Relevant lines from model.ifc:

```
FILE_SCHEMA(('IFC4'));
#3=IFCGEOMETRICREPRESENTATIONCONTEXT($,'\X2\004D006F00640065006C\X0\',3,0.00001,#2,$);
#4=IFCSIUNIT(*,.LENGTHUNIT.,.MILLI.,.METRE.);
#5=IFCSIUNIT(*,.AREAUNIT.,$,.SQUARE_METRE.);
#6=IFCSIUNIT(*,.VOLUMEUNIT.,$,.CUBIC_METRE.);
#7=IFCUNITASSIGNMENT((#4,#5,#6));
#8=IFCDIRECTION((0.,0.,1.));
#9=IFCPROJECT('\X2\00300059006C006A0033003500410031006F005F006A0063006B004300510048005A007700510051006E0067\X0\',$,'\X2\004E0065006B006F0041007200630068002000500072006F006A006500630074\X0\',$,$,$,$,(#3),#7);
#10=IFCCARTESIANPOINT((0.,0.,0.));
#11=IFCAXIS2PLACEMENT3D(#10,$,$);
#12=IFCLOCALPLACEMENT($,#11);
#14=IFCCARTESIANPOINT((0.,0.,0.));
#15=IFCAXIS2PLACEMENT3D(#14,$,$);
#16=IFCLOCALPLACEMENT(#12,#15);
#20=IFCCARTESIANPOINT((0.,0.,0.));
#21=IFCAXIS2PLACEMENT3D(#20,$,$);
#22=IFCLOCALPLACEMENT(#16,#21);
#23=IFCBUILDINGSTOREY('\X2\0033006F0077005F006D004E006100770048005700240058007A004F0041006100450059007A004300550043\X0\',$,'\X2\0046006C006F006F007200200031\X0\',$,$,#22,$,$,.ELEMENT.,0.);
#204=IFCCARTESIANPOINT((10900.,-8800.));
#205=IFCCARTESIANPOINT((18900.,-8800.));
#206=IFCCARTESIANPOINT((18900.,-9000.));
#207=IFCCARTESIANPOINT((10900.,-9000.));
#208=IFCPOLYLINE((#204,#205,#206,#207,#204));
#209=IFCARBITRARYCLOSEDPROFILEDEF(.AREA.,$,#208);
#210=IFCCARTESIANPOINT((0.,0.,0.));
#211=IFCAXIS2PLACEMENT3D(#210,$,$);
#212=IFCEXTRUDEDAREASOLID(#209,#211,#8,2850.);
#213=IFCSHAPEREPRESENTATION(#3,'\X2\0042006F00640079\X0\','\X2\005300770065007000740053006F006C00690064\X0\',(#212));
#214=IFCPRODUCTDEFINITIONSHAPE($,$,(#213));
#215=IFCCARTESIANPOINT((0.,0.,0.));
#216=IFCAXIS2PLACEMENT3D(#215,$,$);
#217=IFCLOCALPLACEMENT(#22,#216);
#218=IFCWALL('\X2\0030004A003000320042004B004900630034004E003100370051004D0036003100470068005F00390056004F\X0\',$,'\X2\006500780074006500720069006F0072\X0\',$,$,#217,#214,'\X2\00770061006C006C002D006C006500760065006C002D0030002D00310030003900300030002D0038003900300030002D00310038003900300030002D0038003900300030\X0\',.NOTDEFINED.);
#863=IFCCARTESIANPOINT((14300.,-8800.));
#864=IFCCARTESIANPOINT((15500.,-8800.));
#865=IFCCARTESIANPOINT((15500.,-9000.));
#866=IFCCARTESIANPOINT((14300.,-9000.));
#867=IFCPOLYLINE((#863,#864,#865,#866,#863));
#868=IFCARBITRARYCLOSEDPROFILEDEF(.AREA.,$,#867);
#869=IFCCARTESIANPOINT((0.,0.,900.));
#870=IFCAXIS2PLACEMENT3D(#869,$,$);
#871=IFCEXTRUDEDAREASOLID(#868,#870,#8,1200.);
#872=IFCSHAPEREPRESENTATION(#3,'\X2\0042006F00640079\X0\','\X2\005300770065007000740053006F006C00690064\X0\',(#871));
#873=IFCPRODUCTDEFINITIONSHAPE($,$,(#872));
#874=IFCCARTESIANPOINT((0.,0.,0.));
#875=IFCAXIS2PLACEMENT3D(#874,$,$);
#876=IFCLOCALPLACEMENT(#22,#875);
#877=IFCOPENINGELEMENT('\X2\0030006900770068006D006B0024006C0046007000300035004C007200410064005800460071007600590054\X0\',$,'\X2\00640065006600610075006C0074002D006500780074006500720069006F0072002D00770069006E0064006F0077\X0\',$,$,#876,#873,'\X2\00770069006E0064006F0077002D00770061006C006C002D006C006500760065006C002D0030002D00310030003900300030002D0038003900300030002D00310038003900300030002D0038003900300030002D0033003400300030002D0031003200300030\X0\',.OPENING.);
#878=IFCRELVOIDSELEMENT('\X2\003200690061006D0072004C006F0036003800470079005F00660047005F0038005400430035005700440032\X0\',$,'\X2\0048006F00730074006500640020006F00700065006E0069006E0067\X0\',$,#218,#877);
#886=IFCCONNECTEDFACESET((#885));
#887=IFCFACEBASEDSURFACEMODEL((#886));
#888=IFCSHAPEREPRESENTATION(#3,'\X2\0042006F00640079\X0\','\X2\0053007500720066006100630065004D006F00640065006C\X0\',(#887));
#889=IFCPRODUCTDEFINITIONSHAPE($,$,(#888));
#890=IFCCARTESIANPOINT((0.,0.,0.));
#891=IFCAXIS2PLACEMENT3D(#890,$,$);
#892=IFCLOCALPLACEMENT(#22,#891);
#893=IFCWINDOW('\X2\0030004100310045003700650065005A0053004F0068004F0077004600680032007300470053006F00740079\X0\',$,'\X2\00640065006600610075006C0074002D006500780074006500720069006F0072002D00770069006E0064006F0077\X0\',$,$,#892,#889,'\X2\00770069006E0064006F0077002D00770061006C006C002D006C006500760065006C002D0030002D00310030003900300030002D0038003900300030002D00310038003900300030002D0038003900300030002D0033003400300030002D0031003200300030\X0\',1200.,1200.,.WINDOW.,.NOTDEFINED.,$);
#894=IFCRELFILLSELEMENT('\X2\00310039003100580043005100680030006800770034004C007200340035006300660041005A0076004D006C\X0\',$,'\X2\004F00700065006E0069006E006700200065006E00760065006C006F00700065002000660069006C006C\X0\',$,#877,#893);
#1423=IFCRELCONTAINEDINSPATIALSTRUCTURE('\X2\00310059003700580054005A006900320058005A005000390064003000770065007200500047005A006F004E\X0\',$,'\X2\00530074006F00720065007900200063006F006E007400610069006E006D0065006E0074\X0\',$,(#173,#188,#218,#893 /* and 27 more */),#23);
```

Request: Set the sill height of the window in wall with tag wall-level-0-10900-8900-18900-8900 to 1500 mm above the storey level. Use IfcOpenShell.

```python
import numpy as np
import ifcopenshell
import ifcopenshell.api.geometry
import ifcopenshell.geom
import ifcopenshell.util.element
import ifcopenshell.util.placement
import ifcopenshell.util.shape
import ifcopenshell.util.unit

model = ifcopenshell.open("model.ifc")
unit_scale = ifcopenshell.util.unit.calculate_unit_scale(model)

window = model.by_guid("0A1E7eeZSOhOwFh2sGSoty")
opening = window.FillsVoids[0].RelatingOpeningElement
storey = ifcopenshell.util.element.get_container(window, ifc_class="IfcBuildingStorey")
level = ifcopenshell.util.placement.get_local_placement(storey.ObjectPlacement)[2, 3]

# The opening's origin need not be at the sill, so measure its lowest point.
shape = ifcopenshell.geom.create_shape(ifcopenshell.geom.settings(), opening)
bottom = ifcopenshell.util.shape.get_shape_bottom_elevation(shape, shape.geometry) / unit_scale
dz = level + 1.5 / unit_scale - bottom

shift = np.array([0.0, 0.0, dz])
# The window is not placed relative to its opening, so move both.
for product in (opening, window):
    matrix = ifcopenshell.util.placement.get_local_placement(product.ObjectPlacement)
    matrix[:3, 3] += shift
    ifcopenshell.api.geometry.edit_object_placement(model, product=product, matrix=matrix, is_si=False)

print(f"moved by {dz * unit_scale:+.3f} m")

model.write("model_edited.ifc")
```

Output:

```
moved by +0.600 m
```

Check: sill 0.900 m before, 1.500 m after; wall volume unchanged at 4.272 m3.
